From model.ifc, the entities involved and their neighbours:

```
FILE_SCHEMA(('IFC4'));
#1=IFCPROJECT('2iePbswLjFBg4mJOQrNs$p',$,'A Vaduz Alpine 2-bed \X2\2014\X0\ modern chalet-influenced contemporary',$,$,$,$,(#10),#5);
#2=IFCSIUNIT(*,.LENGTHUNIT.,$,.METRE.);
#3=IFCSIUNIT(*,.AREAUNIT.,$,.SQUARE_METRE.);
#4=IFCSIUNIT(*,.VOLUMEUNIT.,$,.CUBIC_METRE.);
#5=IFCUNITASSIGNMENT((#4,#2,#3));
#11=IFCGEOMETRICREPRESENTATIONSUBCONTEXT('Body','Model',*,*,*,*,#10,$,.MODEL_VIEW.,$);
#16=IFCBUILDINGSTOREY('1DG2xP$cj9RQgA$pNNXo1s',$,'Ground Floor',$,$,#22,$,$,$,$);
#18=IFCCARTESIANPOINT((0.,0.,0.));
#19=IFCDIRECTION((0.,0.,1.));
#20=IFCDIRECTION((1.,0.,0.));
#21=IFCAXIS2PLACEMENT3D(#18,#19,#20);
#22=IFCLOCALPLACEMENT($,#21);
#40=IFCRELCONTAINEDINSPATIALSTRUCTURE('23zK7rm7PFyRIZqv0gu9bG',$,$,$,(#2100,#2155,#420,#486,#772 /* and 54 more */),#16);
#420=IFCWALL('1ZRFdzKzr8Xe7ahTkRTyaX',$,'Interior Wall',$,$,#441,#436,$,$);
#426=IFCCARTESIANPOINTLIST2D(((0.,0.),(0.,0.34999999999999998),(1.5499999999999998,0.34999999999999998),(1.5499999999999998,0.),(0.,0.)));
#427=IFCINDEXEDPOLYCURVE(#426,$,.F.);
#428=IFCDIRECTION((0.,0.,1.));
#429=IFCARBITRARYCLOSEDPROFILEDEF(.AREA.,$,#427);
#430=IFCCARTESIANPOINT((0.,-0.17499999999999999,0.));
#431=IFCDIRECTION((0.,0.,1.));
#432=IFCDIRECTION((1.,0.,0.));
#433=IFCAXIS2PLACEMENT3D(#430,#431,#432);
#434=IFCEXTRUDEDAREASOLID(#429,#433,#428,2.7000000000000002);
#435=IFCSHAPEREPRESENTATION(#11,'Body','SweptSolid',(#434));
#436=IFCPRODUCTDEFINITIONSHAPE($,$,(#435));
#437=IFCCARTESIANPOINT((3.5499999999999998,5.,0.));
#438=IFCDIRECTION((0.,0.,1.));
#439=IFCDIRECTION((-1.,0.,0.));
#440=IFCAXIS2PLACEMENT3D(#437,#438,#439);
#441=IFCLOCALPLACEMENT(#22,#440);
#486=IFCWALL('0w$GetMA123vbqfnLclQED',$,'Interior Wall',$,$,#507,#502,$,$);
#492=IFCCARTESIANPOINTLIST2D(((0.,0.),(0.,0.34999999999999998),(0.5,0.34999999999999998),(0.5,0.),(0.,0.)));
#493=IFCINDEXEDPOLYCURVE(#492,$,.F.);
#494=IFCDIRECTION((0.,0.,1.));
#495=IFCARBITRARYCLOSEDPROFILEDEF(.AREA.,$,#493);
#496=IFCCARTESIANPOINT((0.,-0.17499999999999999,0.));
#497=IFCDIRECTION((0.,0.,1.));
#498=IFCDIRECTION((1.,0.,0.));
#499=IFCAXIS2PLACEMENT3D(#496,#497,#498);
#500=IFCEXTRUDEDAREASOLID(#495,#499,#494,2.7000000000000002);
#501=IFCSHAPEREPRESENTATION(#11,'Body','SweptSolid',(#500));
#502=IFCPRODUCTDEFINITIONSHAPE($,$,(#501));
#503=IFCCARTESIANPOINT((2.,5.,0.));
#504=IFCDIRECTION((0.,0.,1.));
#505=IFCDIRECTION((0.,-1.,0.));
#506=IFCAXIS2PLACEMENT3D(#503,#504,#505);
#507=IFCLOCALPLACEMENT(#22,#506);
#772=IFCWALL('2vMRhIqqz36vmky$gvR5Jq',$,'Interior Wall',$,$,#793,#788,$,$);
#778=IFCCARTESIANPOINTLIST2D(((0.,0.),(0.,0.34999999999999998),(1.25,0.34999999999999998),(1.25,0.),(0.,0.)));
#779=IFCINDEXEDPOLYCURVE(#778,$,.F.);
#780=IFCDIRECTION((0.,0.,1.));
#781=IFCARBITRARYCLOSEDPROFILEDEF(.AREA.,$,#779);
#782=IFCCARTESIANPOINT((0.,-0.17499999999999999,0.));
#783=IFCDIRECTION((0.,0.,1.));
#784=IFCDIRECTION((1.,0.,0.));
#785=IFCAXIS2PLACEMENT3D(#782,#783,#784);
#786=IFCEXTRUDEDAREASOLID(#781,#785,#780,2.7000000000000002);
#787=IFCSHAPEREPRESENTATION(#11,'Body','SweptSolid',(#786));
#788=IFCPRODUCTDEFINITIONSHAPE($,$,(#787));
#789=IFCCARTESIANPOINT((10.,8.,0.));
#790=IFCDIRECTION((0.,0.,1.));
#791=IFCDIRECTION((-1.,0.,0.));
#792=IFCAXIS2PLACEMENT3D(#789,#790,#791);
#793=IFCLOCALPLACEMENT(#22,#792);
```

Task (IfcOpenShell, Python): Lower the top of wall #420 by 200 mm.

```python
import ifcopenshell
import ifcopenshell.geom
import ifcopenshell.util.representation
import ifcopenshell.util.shape

model = ifcopenshell.open("model.ifc")
settings = ifcopenshell.geom.settings()


def volume(element):
    """Net volume in cubic metres, openings subtracted."""
    shape = ifcopenshell.geom.create_shape(settings, element)
    return ifcopenshell.util.shape.get_volume(shape.geometry)


wall = model.by_id(420)
before = volume(wall)

body = ifcopenshell.util.representation.get_representation(wall, "Model", "Body")
solid = body.Items[0]
old_height = solid.Depth
solid.Depth -= 0.2
after = volume(wall)

print(f"height {old_height:g} -> {solid.Depth:g}, volume {before:.3f} -> {after:.3f} m3")

model.write("model_edited.ifc")
```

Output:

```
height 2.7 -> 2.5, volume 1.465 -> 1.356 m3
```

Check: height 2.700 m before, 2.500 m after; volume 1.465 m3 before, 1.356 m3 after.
